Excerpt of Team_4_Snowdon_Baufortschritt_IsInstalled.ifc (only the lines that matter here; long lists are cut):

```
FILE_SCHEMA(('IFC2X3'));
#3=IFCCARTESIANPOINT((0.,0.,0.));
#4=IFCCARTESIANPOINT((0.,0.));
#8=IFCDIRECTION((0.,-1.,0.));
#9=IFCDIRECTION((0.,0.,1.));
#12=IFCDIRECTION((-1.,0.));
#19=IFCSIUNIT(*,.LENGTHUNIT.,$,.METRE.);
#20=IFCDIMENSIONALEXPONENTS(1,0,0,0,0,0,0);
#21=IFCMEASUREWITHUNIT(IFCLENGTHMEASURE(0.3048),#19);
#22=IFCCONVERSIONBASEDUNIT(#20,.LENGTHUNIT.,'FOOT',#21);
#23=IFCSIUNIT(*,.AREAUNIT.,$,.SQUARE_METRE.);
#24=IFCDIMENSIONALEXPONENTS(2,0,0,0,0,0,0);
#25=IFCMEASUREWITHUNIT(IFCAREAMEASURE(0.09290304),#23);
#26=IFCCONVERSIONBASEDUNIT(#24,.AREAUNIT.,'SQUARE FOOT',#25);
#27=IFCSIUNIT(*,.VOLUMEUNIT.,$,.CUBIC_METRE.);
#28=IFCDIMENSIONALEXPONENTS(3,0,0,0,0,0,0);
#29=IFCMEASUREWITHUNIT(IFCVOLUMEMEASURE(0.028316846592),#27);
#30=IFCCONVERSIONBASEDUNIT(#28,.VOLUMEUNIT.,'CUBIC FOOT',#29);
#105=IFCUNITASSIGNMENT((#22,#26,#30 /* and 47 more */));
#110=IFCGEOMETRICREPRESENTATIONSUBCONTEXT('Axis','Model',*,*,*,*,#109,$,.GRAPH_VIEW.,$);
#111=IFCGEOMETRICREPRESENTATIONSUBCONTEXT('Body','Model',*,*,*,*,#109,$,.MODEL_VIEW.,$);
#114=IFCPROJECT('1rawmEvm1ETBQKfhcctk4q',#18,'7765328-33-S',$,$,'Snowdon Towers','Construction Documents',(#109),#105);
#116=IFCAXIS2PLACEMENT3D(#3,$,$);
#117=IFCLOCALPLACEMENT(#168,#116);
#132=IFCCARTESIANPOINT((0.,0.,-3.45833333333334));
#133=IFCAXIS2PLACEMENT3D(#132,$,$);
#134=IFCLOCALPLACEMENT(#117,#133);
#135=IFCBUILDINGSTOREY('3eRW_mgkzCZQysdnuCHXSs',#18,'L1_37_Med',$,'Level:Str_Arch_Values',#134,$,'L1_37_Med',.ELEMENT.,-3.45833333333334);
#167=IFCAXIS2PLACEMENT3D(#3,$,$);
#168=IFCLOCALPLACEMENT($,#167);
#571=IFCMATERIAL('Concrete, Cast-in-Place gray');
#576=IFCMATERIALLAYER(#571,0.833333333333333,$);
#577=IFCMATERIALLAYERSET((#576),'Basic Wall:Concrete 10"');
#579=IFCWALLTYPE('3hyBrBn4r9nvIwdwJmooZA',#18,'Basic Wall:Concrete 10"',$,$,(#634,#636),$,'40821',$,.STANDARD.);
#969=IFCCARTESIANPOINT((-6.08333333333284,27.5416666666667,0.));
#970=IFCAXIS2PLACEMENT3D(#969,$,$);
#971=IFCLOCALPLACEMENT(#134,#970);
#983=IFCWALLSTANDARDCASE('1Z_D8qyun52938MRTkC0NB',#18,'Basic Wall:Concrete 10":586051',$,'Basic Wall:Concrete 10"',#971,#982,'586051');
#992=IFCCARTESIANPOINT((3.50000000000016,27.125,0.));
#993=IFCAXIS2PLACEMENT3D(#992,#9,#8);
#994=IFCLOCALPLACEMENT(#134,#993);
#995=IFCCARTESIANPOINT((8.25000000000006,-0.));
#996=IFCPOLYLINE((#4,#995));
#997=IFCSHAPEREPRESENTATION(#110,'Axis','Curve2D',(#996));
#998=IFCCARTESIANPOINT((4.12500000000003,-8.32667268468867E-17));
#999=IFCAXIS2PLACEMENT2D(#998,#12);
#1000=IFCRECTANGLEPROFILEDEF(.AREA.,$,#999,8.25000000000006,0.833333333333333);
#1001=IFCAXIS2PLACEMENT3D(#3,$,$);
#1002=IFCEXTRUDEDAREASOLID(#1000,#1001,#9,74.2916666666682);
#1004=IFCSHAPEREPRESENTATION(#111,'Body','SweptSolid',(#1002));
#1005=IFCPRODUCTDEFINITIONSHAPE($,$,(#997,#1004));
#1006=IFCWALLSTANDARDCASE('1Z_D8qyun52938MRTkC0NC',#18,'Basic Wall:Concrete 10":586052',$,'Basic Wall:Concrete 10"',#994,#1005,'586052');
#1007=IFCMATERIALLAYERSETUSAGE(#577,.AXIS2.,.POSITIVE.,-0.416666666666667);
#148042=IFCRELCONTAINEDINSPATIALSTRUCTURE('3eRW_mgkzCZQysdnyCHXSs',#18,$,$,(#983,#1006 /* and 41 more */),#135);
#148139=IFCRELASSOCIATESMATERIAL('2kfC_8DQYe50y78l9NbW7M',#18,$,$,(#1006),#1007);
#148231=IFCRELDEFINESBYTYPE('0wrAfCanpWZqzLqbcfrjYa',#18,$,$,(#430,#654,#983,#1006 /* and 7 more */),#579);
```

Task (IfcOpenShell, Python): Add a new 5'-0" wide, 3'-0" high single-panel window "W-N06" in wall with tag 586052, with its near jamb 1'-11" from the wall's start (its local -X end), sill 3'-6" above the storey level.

```python
import numpy as np
import ifcopenshell
import ifcopenshell.api.feature
import ifcopenshell.api.geometry
import ifcopenshell.api.root
import ifcopenshell.api.spatial
import ifcopenshell.api.type
import ifcopenshell.geom
import ifcopenshell.util.element
import ifcopenshell.util.placement
import ifcopenshell.util.representation
import ifcopenshell.util.shape
import ifcopenshell.util.unit

model = ifcopenshell.open("Team_4_Snowdon_Baufortschritt_IsInstalled.ifc")
unit_scale = ifcopenshell.util.unit.calculate_unit_scale(model)
settings = ifcopenshell.geom.settings()


def volume(element):
    """Net volume in cubic metres, openings subtracted."""
    shape = ifcopenshell.geom.create_shape(settings, element)
    return ifcopenshell.util.shape.get_volume(shape.geometry)


wall = model.by_id(1006)
storey = ifcopenshell.util.element.get_container(wall, ifc_class="IfcBuildingStorey")
context = ifcopenshell.util.representation.get_context(model, "Model", "Body", "MODEL_VIEW")
before = volume(wall)

width, height, from_end, sill = 1.524, 0.9144, 0.5842, 1.0668  # metres

# The wall runs along its own X axis, and the end named is its -X end.
wall_shape = ifcopenshell.geom.create_shape(settings, wall)
x, y, z = ifcopenshell.util.shape.get_vertices(wall_shape.geometry).T
start = x.min() + from_end
face, thickness = float(y.min()), float(y.max() - y.min())
wall_matrix = ifcopenshell.util.placement.get_local_placement(wall.ObjectPlacement)
level = ifcopenshell.util.placement.get_local_placement(storey.ObjectPlacement)[2, 3]


def in_wall(x, y):
    """Placement at x, y metres in the wall's axes, at sill height."""
    matrix = wall_matrix.copy()
    matrix[:, 3] = wall_matrix @ np.array([x / unit_scale, y / unit_scale, 0.0, 1.0])
    matrix[2, 3] = level + sill / unit_scale
    return matrix


# Opening: a box that overshoots both wall faces by 50 mm.
opening = ifcopenshell.api.root.create_entity(model, ifc_class="IfcOpeningElement")
box = ifcopenshell.api.geometry.add_wall_representation(
    model, context=context, length=width, height=height, thickness=thickness + 0.1
)
ifcopenshell.api.geometry.assign_representation(model, product=opening, representation=box)
ifcopenshell.api.geometry.edit_object_placement(model, product=opening, matrix=in_wall(start, face - 0.05), is_si=False)
ifcopenshell.api.feature.add_feature(model, feature=opening, element=wall)

window = ifcopenshell.api.root.create_entity(model, ifc_class="IfcWindow", name="W-N06")
window.OverallWidth, window.OverallHeight = width / unit_scale, height / unit_scale
body = ifcopenshell.api.geometry.add_window_representation(
    model,
    context=context,
    overall_width=window.OverallWidth,
    overall_height=window.OverallHeight,
    partition_type="SINGLE_PANEL",
)
ifcopenshell.api.geometry.assign_representation(model, product=window, representation=body)
ifcopenshell.api.spatial.assign_container(model, products=[window], relating_structure=storey)
fills = ifcopenshell.api.feature.add_filling(model, opening=opening, element=window)
fills.OwnerHistory = window.OwnerHistory  # required in IFC2X3

# IFC2X3 keeps the operation on the window style.
style = ifcopenshell.api.root.create_entity(model, ifc_class="IfcWindowStyle", name="W-N06")
style.OperationType, style.ConstructionType = "SINGLE_PANEL", "NOTDEFINED"
style.ParameterTakesPrecedence = style.Sizeable = False
ifcopenshell.api.type.assign_type(model, related_objects=[window], relating_type=style)

# Centre the window in the wall's thickness.
ifcopenshell.api.geometry.edit_object_placement(model, product=window, matrix=in_wall(start, face), is_si=False)
window_shape = ifcopenshell.geom.create_shape(settings, window)
depth = ifcopenshell.util.shape.get_vertices(window_shape.geometry)[:, 1]
offset = face + thickness / 2 - (depth.min() + depth.max()) / 2
ifcopenshell.api.geometry.edit_object_placement(model, product=window, matrix=in_wall(start, offset), is_si=False)

after = volume(wall)

print(f"wall volume {before:.3f} -> {after:.3f} m3")

model.write("Team_4_Snowdon_Baufortschritt_IsInstalled_edited.ifc")
```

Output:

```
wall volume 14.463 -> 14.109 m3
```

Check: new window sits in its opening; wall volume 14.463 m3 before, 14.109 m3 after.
